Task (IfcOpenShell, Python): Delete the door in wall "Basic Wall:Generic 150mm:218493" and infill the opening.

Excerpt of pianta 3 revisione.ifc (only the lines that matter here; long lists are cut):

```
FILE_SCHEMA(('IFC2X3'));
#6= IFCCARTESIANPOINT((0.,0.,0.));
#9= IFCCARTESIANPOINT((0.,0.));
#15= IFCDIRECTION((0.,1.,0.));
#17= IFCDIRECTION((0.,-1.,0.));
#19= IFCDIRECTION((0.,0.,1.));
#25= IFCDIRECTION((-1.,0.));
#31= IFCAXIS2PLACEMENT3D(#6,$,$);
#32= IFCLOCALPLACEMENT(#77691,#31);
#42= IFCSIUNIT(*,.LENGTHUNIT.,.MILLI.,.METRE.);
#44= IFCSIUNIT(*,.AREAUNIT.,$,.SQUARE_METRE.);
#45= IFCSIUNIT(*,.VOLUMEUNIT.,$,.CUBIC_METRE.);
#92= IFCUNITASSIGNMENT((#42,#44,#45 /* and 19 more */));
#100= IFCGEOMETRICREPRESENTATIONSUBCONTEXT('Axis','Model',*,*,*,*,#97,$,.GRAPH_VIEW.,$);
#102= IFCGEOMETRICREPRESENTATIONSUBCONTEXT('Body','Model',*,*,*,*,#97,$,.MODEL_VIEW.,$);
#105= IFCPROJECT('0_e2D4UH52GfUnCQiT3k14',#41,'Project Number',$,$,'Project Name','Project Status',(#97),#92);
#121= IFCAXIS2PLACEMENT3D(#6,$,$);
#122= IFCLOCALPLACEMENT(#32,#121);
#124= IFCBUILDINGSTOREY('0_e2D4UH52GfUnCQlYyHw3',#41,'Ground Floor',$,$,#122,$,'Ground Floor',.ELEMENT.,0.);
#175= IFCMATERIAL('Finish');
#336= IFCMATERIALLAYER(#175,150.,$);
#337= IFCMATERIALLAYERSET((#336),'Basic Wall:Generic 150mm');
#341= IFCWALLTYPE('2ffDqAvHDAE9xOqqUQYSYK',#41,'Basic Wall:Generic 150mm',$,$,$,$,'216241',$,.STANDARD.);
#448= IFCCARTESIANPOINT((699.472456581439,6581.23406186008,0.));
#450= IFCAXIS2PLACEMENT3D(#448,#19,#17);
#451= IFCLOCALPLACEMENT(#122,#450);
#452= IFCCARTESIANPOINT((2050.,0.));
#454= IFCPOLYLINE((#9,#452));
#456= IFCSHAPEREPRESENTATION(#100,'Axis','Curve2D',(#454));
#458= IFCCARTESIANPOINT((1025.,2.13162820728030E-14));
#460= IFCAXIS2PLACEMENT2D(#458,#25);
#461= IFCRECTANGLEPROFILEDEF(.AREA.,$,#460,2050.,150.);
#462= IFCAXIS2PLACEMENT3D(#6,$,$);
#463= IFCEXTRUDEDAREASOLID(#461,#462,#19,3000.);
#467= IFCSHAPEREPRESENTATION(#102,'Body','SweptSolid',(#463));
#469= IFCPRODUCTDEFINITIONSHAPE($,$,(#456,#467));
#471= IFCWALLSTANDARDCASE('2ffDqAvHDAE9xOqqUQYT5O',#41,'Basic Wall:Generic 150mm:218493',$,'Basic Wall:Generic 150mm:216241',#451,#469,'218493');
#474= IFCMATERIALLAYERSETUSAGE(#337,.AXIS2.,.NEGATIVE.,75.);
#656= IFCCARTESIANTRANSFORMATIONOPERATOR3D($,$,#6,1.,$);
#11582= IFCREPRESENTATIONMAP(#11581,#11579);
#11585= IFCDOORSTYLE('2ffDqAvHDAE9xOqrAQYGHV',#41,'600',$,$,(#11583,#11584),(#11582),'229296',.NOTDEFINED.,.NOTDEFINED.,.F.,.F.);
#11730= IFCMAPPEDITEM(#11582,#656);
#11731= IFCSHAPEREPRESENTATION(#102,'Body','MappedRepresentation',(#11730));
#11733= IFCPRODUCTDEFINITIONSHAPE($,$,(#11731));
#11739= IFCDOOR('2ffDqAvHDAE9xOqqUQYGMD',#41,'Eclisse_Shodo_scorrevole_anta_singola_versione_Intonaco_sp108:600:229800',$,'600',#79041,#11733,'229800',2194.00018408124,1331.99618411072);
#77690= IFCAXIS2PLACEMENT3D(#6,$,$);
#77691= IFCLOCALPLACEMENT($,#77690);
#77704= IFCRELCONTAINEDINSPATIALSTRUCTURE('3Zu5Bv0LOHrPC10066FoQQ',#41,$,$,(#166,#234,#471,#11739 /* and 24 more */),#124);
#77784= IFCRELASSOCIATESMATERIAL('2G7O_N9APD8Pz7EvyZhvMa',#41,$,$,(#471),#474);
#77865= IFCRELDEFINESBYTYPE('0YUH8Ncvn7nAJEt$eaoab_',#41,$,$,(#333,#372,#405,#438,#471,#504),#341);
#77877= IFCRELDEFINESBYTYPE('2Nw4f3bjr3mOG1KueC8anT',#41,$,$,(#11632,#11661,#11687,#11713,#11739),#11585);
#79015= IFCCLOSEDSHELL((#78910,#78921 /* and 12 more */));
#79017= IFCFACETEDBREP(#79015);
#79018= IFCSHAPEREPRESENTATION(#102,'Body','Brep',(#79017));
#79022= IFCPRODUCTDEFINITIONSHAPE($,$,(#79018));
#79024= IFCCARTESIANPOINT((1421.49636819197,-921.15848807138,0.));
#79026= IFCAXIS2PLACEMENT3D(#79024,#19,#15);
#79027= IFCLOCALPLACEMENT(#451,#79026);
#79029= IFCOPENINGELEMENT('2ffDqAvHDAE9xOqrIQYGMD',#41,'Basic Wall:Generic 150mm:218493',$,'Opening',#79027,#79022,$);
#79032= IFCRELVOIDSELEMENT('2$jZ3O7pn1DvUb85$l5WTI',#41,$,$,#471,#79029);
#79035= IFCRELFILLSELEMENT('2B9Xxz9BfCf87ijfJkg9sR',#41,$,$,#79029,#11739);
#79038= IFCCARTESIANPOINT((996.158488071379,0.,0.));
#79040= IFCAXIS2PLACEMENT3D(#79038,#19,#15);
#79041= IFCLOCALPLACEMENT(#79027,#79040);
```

```python
import ifcopenshell
import ifcopenshell.api.feature
import ifcopenshell.api.root
import ifcopenshell.geom
import ifcopenshell.util.shape

model = ifcopenshell.open("pianta 3 revisione.ifc")
settings = ifcopenshell.geom.settings()


def volume(element):
    """Net volume in cubic metres, openings subtracted."""
    shape = ifcopenshell.geom.create_shape(settings, element)
    return ifcopenshell.util.shape.get_volume(shape.geometry)


door = model.by_id(11739)
opening = door.FillsVoids[0].RelatingOpeningElement
wall = opening.VoidsElements[0].RelatingBuildingElement
before = volume(wall)

ifcopenshell.api.root.remove_product(model, product=door)
ifcopenshell.api.feature.remove_feature(model, feature=opening)

after = volume(wall)

print(f"wall volume {before:.3f} -> {after:.3f} m3")

model.write("pianta 3 revisione-out.ifc")
```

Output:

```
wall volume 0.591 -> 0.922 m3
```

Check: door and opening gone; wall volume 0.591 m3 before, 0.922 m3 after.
